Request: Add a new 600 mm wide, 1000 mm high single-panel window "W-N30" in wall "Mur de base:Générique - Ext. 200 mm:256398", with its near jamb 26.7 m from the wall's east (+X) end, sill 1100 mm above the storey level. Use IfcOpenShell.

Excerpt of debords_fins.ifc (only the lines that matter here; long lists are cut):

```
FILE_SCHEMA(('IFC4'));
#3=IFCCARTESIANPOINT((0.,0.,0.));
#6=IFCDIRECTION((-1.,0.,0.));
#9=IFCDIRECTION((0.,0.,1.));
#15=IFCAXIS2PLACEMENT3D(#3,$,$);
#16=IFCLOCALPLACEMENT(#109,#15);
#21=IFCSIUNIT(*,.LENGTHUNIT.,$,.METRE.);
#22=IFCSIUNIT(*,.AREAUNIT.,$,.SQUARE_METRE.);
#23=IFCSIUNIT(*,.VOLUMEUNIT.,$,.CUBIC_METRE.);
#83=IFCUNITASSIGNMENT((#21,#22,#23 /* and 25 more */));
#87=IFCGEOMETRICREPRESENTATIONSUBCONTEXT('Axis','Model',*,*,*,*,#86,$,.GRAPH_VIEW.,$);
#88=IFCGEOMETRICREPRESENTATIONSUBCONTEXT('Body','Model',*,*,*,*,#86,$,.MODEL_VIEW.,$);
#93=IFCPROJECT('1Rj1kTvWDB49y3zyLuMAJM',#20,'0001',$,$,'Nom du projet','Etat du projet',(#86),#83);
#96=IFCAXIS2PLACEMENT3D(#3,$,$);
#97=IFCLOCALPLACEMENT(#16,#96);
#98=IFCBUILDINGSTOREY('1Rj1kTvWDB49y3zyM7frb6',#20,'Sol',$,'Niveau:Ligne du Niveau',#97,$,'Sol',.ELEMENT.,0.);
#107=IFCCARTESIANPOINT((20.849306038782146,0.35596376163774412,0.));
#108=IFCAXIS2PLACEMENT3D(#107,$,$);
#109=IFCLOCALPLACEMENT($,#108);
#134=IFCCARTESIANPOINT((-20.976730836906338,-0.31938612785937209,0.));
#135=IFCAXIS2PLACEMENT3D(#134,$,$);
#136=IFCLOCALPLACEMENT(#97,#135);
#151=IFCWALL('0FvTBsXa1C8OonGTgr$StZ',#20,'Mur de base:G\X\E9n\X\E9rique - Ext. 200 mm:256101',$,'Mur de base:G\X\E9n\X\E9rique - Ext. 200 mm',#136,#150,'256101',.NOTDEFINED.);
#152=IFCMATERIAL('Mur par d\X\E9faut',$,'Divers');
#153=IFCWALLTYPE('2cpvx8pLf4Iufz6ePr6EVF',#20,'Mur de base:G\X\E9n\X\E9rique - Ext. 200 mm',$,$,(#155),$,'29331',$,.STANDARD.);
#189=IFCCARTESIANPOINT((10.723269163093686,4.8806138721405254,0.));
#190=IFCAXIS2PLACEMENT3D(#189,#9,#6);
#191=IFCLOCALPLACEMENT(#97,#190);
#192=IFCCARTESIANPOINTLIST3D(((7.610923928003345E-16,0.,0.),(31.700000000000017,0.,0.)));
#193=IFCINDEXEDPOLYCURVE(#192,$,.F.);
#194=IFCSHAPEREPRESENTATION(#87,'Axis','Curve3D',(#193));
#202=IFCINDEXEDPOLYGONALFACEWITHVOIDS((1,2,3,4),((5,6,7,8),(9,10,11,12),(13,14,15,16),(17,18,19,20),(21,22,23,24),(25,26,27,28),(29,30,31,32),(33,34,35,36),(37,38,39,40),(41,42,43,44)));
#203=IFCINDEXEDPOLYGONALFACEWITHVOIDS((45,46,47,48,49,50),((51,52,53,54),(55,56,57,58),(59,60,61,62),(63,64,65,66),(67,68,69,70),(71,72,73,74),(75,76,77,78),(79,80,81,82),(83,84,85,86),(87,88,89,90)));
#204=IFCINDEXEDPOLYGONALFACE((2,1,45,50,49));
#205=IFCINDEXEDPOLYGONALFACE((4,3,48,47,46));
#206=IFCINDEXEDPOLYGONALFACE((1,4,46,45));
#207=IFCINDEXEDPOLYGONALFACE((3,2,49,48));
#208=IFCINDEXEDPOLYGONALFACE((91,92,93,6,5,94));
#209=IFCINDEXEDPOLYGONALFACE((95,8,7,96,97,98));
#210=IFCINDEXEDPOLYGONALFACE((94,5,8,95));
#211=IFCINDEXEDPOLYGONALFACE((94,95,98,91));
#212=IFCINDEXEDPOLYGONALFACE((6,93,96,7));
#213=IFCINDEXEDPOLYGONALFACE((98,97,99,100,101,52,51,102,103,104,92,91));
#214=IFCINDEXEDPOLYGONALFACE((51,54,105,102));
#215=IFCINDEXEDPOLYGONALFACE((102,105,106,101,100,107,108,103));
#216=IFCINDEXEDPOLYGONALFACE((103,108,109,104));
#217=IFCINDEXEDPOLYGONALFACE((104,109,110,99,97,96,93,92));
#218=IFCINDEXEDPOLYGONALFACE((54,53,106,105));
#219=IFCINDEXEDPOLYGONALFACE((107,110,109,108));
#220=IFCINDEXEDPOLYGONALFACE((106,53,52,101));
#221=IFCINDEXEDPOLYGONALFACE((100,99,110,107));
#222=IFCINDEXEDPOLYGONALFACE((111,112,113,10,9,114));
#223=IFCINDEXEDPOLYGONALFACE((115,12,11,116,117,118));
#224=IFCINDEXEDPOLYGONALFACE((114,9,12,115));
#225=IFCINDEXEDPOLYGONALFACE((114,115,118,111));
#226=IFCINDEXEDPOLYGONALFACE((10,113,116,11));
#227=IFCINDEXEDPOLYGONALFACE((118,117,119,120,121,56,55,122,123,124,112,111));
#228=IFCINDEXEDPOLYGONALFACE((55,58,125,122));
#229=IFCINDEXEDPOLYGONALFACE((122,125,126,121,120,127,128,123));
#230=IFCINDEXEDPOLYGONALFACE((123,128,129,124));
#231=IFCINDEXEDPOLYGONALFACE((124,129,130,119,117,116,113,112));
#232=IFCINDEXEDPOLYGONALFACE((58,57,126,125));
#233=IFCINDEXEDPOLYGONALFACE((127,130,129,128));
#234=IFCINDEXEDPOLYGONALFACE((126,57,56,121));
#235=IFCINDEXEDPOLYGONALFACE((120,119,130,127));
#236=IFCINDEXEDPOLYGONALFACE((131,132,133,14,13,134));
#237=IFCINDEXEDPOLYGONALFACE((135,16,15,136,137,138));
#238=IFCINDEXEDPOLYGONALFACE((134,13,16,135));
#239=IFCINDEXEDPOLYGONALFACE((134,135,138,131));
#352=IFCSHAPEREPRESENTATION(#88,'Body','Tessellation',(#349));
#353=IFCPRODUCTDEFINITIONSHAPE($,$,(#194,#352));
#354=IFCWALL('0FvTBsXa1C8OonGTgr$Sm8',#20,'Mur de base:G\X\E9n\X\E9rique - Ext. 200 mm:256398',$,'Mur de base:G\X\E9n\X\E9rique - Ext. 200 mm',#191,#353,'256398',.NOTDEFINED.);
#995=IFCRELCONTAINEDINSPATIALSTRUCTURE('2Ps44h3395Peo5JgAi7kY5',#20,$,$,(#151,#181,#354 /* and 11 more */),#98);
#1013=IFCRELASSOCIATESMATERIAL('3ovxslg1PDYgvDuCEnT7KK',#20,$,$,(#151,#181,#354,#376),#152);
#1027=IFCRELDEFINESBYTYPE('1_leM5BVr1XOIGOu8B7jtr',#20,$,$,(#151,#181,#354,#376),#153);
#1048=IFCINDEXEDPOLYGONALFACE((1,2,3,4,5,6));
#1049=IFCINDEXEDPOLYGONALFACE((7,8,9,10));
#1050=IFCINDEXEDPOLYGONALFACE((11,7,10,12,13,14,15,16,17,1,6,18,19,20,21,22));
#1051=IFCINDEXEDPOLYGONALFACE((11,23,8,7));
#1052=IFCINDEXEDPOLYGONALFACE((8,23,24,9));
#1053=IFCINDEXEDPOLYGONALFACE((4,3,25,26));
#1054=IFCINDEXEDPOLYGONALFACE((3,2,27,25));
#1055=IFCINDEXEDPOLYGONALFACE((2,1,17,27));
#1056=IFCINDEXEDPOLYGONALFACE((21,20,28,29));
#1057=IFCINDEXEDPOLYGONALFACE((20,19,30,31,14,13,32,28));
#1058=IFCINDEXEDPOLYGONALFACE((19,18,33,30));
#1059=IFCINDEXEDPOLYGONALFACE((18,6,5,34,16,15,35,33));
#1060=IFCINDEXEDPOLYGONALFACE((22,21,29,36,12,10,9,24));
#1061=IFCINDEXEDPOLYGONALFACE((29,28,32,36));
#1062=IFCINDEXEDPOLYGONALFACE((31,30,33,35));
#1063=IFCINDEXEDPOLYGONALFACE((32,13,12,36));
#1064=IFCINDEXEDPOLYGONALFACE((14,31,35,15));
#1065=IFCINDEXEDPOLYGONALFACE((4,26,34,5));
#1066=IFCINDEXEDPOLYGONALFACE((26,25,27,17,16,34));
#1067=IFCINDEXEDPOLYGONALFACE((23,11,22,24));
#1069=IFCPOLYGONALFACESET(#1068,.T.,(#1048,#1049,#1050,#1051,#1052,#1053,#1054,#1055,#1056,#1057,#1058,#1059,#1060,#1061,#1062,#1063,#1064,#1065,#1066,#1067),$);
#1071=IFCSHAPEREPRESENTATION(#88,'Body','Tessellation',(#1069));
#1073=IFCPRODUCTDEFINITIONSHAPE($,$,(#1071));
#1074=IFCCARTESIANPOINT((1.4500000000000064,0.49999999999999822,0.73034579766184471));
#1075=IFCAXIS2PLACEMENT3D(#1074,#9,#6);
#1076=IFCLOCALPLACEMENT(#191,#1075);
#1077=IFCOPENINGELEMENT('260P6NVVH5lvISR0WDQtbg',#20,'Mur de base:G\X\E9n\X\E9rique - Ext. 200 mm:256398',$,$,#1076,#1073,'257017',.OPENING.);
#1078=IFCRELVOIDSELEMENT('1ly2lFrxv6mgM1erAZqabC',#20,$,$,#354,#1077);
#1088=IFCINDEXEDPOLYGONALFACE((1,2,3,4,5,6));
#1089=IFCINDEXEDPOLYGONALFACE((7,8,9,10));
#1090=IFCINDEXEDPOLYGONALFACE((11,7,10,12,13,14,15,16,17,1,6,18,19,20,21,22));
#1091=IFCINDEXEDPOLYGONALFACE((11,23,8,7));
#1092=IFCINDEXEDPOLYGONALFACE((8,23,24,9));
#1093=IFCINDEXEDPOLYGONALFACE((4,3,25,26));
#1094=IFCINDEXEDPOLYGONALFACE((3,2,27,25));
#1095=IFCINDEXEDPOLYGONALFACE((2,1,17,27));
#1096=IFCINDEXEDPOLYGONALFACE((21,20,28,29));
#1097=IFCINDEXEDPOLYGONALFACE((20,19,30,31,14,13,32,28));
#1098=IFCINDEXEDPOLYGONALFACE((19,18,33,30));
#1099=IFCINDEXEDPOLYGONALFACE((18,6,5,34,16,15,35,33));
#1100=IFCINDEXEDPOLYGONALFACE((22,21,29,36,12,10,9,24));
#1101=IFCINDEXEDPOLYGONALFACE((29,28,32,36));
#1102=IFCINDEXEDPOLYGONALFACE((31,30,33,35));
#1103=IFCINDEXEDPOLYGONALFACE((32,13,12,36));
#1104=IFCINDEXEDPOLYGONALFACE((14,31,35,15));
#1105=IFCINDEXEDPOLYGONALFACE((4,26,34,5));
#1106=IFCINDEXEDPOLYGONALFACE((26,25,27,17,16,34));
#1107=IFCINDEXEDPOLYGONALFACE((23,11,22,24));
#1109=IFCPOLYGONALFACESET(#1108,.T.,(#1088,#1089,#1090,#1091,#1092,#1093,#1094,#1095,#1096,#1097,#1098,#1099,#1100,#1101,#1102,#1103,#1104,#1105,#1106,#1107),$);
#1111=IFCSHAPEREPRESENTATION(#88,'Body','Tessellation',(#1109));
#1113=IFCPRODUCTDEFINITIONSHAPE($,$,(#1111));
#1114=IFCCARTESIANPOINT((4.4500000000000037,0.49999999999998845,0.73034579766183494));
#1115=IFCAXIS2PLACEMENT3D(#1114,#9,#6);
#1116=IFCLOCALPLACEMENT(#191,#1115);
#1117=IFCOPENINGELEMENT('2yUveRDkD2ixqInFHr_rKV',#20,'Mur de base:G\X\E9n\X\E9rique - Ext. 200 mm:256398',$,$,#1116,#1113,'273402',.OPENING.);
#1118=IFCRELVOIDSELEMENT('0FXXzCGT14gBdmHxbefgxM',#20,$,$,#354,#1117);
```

```python
import numpy as np
import ifcopenshell
import ifcopenshell.api.feature
import ifcopenshell.api.geometry
import ifcopenshell.api.root
import ifcopenshell.api.spatial
import ifcopenshell.geom
import ifcopenshell.util.element
import ifcopenshell.util.placement
import ifcopenshell.util.representation
import ifcopenshell.util.shape
import ifcopenshell.util.unit

model = ifcopenshell.open("debords_fins.ifc")
unit_scale = ifcopenshell.util.unit.calculate_unit_scale(model)
settings = ifcopenshell.geom.settings()


def volume(element):
    """Net volume in cubic metres, openings subtracted."""
    shape = ifcopenshell.geom.create_shape(settings, element)
    return ifcopenshell.util.shape.get_volume(shape.geometry)


wall = model.by_guid("0FvTBsXa1C8OonGTgr$Sm8")
storey = ifcopenshell.util.element.get_container(wall, ifc_class="IfcBuildingStorey")
context = ifcopenshell.util.representation.get_context(model, "Model", "Body", "MODEL_VIEW")
before = volume(wall)

width, height, from_end, sill = 0.6, 1, 26.7, 1.1  # metres

# The wall runs along its own X axis, and the end named is its -X end.
wall_shape = ifcopenshell.geom.create_shape(settings, wall)
x, y, z = ifcopenshell.util.shape.get_vertices(wall_shape.geometry).T
start = x.min() + from_end
face, thickness = float(y.min()), float(y.max() - y.min())
wall_matrix = ifcopenshell.util.placement.get_local_placement(wall.ObjectPlacement)
level = ifcopenshell.util.placement.get_local_placement(storey.ObjectPlacement)[2, 3]


def in_wall(x, y):
    """Placement at x, y metres in the wall's axes, at sill height."""
    matrix = wall_matrix.copy()
    matrix[:, 3] = wall_matrix @ np.array([x / unit_scale, y / unit_scale, 0.0, 1.0])
    matrix[2, 3] = level + sill / unit_scale
    return matrix


# Opening: a box that overshoots both wall faces by 50 mm.
opening = ifcopenshell.api.root.create_entity(model, ifc_class="IfcOpeningElement", predefined_type="OPENING")
box = ifcopenshell.api.geometry.add_wall_representation(
    model, context=context, length=width, height=height, thickness=thickness + 0.1
)
ifcopenshell.api.geometry.assign_representation(model, product=opening, representation=box)
ifcopenshell.api.geometry.edit_object_placement(model, product=opening, matrix=in_wall(start, face - 0.05), is_si=False)
ifcopenshell.api.feature.add_feature(model, feature=opening, element=wall)

window = ifcopenshell.api.root.create_entity(model, ifc_class="IfcWindow", name="W-N30", predefined_type="WINDOW")
window.OverallWidth, window.OverallHeight = width / unit_scale, height / unit_scale
window.PartitioningType = "SINGLE_PANEL"
body = ifcopenshell.api.geometry.add_window_representation(
    model,
    context=context,
    overall_width=window.OverallWidth,
    overall_height=window.OverallHeight,
    partition_type="SINGLE_PANEL",
)
ifcopenshell.api.geometry.assign_representation(model, product=window, representation=body)
ifcopenshell.api.spatial.assign_container(model, products=[window], relating_structure=storey)
ifcopenshell.api.feature.add_filling(model, opening=opening, element=window)

# Centre the window in the wall's thickness.
ifcopenshell.api.geometry.edit_object_placement(model, product=window, matrix=in_wall(start, face), is_si=False)
window_shape = ifcopenshell.geom.create_shape(settings, window)
depth = ifcopenshell.util.shape.get_vertices(window_shape.geometry)[:, 1]
offset = face + thickness / 2 - (depth.min() + depth.max()) / 2
ifcopenshell.api.geometry.edit_object_placement(model, product=window, matrix=in_wall(start, offset), is_si=False)

after = volume(wall)

print(f"wall volume {before:.3f} -> {after:.3f} m3")

model.write("debords_fins_edited.ifc")
```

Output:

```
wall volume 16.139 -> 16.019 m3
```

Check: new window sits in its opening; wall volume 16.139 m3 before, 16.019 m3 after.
